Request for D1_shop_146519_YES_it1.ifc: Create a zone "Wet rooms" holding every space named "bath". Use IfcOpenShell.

First a look at what the model holds.

```python
import ifcopenshell

model = ifcopenshell.open("D1_shop_146519_YES_it1.ifc")
print(model.schema)
seen = {}
for space in model.by_type("IfcSpace"):
    seen[space.LongName] = seen.get(space.LongName, 0) + 1
for name, count in sorted(seen.items(), key=str):
    print(count, "x", name)
print("zones:", [z.Name for z in model.by_type("IfcZone")][:20])
```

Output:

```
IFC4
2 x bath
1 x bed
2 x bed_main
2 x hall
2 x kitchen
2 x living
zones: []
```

```python
import ifcopenshell
import ifcopenshell.api.group
import ifcopenshell.api.root

model = ifcopenshell.open("D1_shop_146519_YES_it1.ifc")

names = {"bath"}
spaces = [s for s in model.by_type("IfcSpace") if s.LongName in names]

zone = ifcopenshell.api.root.create_entity(model, ifc_class="IfcZone", name="Wet rooms")
ifcopenshell.api.group.assign_group(model, products=spaces, group=zone)
print(len(spaces), "spaces in", zone.Name)

model.write("D1_shop_146519_YES_it1_rev.ifc")
```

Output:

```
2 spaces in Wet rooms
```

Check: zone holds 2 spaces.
